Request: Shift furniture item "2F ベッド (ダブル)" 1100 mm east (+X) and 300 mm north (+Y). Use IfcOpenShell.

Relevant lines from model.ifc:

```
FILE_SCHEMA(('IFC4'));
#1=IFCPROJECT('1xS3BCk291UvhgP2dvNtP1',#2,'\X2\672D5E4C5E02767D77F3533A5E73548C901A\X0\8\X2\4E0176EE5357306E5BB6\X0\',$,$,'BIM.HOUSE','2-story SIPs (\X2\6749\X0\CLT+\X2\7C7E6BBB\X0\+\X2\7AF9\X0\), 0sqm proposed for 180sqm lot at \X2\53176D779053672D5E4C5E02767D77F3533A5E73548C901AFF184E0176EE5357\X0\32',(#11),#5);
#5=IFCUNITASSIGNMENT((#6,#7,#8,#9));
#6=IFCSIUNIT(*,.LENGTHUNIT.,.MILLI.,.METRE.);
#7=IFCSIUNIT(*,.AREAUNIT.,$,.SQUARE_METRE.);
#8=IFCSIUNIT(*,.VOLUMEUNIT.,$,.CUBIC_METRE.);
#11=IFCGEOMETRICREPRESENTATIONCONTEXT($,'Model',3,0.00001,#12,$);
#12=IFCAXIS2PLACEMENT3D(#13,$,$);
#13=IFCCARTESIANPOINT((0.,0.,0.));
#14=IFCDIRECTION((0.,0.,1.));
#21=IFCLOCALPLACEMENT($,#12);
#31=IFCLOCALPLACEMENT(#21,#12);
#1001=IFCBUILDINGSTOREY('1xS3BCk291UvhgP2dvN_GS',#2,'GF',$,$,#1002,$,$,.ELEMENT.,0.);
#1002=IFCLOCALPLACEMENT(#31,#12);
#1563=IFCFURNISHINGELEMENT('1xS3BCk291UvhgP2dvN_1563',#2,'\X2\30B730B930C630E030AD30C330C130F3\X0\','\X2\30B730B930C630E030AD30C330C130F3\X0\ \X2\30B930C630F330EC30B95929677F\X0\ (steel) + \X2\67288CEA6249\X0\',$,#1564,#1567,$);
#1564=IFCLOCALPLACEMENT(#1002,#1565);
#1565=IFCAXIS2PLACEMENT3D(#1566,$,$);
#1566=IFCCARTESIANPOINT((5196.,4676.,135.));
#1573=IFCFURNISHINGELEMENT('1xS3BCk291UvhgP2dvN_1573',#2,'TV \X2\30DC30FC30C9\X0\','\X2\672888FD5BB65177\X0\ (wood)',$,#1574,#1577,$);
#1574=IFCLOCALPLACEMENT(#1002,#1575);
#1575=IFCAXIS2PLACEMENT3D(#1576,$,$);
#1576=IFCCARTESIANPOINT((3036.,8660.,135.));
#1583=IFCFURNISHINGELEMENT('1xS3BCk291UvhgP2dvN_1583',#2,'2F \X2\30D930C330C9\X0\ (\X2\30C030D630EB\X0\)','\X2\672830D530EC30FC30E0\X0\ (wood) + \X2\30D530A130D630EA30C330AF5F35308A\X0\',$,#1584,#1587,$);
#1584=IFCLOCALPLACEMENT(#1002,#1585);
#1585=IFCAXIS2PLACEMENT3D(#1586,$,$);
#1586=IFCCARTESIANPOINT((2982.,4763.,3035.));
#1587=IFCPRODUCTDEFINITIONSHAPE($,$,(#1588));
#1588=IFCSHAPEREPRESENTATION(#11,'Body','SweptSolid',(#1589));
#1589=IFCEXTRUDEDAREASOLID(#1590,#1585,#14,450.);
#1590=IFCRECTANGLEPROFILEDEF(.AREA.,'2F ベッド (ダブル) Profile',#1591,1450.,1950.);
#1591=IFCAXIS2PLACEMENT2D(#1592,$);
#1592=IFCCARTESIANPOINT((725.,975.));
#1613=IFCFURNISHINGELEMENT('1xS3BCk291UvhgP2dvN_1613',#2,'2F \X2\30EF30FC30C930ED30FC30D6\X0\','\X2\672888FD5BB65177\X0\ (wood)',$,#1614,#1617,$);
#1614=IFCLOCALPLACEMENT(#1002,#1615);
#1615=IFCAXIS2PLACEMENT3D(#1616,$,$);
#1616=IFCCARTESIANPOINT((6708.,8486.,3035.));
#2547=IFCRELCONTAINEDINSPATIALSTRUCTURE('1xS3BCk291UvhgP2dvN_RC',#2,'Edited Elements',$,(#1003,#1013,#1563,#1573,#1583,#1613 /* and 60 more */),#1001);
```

```python
import ifcopenshell
import ifcopenshell.api.geometry
import ifcopenshell.util.placement
import ifcopenshell.util.unit

model = ifcopenshell.open("model.ifc")
unit_scale = ifcopenshell.util.unit.calculate_unit_scale(model)

item = model.by_guid("1xS3BCk291UvhgP2dvN_1583")
matrix = ifcopenshell.util.placement.get_local_placement(item.ObjectPlacement)
matrix[0, 3] += 1.1 / unit_scale
matrix[1, 3] += 0.3 / unit_scale
ifcopenshell.api.geometry.edit_object_placement(model, product=item, matrix=matrix, is_si=False)

print(ifcopenshell.util.placement.get_local_placement(item.ObjectPlacement).round(3) + 0.0)

model.write("model_rev.ifc")
```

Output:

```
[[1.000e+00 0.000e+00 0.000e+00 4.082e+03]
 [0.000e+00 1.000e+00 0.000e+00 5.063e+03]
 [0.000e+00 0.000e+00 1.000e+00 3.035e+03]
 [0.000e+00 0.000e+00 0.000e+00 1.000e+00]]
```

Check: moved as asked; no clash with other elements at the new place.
